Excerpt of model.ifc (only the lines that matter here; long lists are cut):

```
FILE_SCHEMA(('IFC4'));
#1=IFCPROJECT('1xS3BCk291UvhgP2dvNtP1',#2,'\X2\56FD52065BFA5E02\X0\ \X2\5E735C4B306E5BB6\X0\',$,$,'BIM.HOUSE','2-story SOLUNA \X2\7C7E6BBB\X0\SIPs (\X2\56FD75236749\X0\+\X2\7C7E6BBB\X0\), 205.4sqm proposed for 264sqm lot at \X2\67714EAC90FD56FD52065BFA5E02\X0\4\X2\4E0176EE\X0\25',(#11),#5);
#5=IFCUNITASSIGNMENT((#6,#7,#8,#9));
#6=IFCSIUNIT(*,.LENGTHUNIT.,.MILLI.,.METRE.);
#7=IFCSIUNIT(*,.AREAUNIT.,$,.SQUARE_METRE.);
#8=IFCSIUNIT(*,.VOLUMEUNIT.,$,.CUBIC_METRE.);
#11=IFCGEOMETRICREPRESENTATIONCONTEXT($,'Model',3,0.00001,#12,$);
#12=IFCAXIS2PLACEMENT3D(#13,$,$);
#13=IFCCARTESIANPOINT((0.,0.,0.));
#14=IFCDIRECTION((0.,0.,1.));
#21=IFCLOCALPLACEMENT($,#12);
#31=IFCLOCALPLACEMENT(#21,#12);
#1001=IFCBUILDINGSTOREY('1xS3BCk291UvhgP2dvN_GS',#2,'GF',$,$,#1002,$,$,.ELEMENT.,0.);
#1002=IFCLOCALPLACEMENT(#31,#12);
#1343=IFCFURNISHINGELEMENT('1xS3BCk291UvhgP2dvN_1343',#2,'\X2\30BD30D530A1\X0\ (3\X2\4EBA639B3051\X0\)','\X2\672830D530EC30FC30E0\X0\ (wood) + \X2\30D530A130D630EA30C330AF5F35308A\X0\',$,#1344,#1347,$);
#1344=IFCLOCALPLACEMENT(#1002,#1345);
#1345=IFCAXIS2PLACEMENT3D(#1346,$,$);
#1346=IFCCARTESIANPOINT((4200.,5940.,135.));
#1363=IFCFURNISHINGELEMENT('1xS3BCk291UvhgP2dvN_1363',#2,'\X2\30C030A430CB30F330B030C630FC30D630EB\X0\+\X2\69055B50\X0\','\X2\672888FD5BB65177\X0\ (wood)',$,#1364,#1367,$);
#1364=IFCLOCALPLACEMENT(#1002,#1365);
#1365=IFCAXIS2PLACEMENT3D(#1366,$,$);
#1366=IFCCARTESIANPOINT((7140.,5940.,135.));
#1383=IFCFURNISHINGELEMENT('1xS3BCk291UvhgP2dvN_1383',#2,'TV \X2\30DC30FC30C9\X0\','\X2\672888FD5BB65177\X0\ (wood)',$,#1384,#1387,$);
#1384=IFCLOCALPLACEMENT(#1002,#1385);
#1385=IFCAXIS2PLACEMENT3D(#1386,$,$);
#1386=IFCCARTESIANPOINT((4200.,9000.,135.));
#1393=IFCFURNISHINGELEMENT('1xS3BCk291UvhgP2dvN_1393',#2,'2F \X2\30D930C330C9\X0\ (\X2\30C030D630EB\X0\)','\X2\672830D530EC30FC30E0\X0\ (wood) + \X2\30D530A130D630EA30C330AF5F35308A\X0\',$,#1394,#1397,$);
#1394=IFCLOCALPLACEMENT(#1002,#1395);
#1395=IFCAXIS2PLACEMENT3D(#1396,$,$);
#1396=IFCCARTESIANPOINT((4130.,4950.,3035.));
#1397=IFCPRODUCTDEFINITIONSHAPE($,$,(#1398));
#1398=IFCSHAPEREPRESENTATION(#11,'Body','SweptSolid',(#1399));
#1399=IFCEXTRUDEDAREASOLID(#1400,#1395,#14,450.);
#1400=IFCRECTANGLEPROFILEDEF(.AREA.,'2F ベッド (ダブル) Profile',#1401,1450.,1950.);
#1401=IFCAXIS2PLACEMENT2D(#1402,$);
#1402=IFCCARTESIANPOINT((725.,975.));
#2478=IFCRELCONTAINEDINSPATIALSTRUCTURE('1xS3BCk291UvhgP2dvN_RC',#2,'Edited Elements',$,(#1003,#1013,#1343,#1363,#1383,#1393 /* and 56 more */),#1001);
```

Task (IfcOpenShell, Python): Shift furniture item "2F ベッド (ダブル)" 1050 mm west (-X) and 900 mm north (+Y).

```python
import ifcopenshell
import ifcopenshell.api.geometry
import ifcopenshell.util.placement

model = ifcopenshell.open("model.ifc")

item = model.by_guid("1xS3BCk291UvhgP2dvN_1393")
matrix = ifcopenshell.util.placement.get_local_placement(item.ObjectPlacement)
matrix[0, 3] -= 1050.0
matrix[1, 3] += 900.0
ifcopenshell.api.geometry.edit_object_placement(model, product=item, matrix=matrix, is_si=False)

print(ifcopenshell.util.placement.get_local_placement(item.ObjectPlacement).round(3) + 0.0)

model.write("model_v2.ifc")
```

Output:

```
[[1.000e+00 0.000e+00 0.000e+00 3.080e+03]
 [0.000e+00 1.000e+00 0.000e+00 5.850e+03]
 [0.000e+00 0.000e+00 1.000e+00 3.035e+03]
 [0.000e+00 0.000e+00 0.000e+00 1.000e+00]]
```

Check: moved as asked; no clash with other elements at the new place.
